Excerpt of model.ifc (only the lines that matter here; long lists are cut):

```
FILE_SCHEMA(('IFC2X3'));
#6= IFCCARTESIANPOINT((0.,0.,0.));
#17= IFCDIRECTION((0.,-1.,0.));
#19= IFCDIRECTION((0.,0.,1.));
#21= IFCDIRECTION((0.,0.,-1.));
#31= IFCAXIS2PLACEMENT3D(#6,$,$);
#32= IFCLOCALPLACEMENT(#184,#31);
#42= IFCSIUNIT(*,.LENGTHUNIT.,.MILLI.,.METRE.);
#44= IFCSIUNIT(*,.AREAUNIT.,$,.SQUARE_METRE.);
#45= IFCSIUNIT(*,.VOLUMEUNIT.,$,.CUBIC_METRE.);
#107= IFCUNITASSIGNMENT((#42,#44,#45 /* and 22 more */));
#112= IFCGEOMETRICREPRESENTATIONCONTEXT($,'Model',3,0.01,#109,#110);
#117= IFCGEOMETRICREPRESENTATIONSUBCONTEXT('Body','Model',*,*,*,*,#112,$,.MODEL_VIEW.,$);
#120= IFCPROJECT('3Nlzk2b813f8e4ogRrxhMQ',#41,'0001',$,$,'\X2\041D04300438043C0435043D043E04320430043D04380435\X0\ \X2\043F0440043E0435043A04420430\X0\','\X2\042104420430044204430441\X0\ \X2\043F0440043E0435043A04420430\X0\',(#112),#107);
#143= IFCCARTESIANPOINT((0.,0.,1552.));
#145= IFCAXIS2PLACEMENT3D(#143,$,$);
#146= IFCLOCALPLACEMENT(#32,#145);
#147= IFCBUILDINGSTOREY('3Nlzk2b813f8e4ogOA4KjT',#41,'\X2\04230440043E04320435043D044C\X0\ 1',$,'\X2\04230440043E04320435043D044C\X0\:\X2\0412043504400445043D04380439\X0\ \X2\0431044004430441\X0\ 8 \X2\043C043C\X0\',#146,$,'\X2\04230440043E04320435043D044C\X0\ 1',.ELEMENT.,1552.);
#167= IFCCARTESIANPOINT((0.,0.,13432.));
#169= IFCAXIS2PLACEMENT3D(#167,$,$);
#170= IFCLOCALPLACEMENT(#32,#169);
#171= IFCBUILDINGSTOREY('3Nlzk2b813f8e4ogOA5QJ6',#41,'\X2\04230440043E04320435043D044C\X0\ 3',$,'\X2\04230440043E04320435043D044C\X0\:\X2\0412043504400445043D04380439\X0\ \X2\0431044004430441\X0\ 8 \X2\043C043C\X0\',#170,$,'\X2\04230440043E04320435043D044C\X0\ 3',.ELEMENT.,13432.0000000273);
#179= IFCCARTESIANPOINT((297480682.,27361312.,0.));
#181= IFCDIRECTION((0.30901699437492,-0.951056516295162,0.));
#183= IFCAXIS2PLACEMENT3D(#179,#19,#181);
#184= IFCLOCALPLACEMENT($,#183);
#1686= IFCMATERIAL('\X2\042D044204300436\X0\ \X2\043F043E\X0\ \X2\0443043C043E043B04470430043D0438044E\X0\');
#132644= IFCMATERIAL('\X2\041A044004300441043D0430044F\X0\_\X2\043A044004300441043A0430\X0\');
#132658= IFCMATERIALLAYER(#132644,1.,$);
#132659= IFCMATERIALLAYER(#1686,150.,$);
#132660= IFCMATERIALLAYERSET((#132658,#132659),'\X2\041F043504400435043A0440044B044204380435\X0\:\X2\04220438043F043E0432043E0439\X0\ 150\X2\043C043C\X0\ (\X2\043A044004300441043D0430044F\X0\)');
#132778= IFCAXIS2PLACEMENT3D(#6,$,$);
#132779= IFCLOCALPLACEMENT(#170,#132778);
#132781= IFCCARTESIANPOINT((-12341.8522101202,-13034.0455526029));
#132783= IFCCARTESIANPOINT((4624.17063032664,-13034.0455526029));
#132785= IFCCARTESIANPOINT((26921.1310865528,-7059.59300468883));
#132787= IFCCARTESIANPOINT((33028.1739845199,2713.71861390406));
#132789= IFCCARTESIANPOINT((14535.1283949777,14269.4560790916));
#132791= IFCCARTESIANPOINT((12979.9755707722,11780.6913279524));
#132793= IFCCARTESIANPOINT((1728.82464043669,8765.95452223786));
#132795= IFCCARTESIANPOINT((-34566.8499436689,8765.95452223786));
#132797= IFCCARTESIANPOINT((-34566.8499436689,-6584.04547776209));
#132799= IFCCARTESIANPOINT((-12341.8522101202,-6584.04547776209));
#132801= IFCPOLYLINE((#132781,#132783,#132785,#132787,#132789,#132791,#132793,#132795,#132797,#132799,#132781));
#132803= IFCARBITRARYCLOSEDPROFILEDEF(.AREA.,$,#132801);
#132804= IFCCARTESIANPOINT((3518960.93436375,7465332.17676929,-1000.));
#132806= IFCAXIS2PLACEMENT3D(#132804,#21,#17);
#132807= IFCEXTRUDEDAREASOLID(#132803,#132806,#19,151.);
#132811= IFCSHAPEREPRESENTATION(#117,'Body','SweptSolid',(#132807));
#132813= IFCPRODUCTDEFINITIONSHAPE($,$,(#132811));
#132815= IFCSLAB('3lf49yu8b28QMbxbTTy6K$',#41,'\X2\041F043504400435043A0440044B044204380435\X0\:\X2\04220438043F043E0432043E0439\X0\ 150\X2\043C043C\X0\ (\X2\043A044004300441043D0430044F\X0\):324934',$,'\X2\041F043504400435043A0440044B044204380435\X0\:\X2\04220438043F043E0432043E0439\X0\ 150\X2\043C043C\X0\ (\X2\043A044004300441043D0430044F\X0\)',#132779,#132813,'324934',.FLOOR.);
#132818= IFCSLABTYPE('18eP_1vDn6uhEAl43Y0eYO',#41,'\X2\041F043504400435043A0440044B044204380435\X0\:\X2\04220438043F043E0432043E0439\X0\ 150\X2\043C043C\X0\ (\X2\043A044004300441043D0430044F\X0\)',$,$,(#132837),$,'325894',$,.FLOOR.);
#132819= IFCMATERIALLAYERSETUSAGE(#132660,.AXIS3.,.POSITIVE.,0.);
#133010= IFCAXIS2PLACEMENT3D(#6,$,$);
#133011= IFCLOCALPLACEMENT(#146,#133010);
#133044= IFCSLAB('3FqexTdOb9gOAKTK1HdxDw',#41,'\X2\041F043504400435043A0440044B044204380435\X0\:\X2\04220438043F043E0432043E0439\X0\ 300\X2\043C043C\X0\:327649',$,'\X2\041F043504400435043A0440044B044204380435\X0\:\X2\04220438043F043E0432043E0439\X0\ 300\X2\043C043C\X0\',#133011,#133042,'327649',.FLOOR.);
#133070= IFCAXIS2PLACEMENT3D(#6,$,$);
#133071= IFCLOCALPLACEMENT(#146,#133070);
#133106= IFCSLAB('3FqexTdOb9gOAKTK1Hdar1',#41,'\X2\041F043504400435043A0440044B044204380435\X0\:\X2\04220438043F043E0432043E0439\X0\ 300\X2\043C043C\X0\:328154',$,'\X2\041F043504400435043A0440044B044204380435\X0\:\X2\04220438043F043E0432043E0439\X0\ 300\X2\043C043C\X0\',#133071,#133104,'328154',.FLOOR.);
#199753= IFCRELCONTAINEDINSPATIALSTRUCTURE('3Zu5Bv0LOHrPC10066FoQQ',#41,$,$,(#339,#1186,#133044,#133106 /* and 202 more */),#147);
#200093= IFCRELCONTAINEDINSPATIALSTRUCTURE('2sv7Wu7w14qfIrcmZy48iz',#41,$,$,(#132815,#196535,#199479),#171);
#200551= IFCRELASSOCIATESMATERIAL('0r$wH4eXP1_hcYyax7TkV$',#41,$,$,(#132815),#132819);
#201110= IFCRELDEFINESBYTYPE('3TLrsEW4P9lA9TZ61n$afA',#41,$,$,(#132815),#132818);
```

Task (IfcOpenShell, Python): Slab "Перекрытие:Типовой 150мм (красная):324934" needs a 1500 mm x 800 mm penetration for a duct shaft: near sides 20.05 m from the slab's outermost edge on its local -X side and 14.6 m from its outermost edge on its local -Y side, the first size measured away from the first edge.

```python
import numpy as np
import ifcopenshell
import ifcopenshell.api.feature
import ifcopenshell.api.geometry
import ifcopenshell.api.root
import ifcopenshell.geom
import ifcopenshell.util.placement
import ifcopenshell.util.representation
import ifcopenshell.util.shape
import ifcopenshell.util.unit

model = ifcopenshell.open("model.ifc")
unit_scale = ifcopenshell.util.unit.calculate_unit_scale(model)
settings = ifcopenshell.geom.settings()


def volume(element):
    """Net volume in cubic metres, openings subtracted."""
    shape = ifcopenshell.geom.create_shape(settings, element)
    return ifcopenshell.util.shape.get_volume(shape.geometry)


slab = model.by_guid("3lf49yu8b28QMbxbTTy6K$")
before = volume(slab)

# Extent in the slab's own axes, in metres. The edges named are its -X and -Y sides.
slab_shape = ifcopenshell.geom.create_shape(settings, slab)
vertices = ifcopenshell.util.shape.get_vertices(slab_shape.geometry)
x_min, y_min, bottom = vertices.min(axis=0)
top = vertices[:, 2].max()

opening = ifcopenshell.api.root.create_entity(model, ifc_class="IfcOpeningElement", name="Duct shaft opening")
context = ifcopenshell.util.representation.get_context(model, "Model", "Body", "MODEL_VIEW")
width, depth = 1.5, 0.8
outline = [(0.0, 0.0), (width, 0.0), (width, depth), (0.0, depth), (0.0, 0.0)]
# Overshoot both faces by 50 mm so the cut is clean.
shape = ifcopenshell.api.geometry.add_slab_representation(
    model, context=context, depth=top - bottom + 0.1, polyline=outline
)
ifcopenshell.api.geometry.assign_representation(model, product=opening, representation=shape)

matrix = ifcopenshell.util.placement.get_local_placement(slab.ObjectPlacement)
matrix[:, 3] = matrix @ np.append(np.array([x_min + 20.05, y_min + 14.6, bottom - 0.05]) / unit_scale, 1.0)
ifcopenshell.api.geometry.edit_object_placement(model, product=opening, matrix=matrix, is_si=False)
ifcopenshell.api.feature.add_feature(model, feature=opening, element=slab)

after = volume(slab)

print(f"slab volume {before:.3f} -> {after:.3f} m3")

model.write("model_rev.ifc")
```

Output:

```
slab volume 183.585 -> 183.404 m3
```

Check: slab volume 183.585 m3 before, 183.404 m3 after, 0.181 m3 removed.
